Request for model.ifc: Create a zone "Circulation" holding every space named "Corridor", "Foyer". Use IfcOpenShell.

First a look at what the model holds.

```python
import ifcopenshell

model = ifcopenshell.open("model.ifc")
print(model.schema)
seen = {}
for space in model.by_type("IfcSpace"):
    seen[space.LongName] = seen.get(space.LongName, 0) + 1
for name, count in sorted(seen.items(), key=str):
    print(count, "x", name)
print("zones:", [z.Name for z in model.by_type("IfcZone")][:20])
```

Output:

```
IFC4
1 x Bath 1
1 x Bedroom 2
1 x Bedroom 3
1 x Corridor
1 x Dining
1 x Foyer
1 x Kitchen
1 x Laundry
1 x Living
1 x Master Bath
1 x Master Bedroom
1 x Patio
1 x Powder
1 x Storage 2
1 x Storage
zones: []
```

```python
import ifcopenshell
import ifcopenshell.api.group
import ifcopenshell.api.root

model = ifcopenshell.open("model.ifc")

names = {"Corridor", "Foyer"}
spaces = [s for s in model.by_type("IfcSpace") if s.LongName in names]

zone = ifcopenshell.api.root.create_entity(model, ifc_class="IfcZone", name="Circulation")
ifcopenshell.api.group.assign_group(model, products=spaces, group=zone)
print(len(spaces), "spaces in", zone.Name)

model.write("model_rev.ifc")
```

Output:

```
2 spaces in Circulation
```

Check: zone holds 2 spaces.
